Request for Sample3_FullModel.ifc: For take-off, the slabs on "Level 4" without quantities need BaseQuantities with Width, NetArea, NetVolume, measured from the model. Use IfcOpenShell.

First a look at what the model holds.

```python
import ifcopenshell
import ifcopenshell.util.element
import ifcopenshell.util.unit

model = ifcopenshell.open("Sample3_FullModel.ifc")
print(model.schema)
for unit_type in ("LENGTHUNIT", "AREAUNIT", "VOLUMEUNIT"):
    print(unit_type, ifcopenshell.util.unit.calculate_unit_scale(model, unit_type))
storey = next(s for s in model.by_type("IfcBuildingStorey") if s.Name == "Level 4")
slabs = [e for e in ifcopenshell.util.element.get_decomposition(storey) if e.is_a("IfcSlab")]
for e in sorted(slabs, key=lambda e: e.id()):
    print(e.id(), e.is_a(), e.Name, list(ifcopenshell.util.element.get_psets(e, qtos_only=True)), sep=" | ")
```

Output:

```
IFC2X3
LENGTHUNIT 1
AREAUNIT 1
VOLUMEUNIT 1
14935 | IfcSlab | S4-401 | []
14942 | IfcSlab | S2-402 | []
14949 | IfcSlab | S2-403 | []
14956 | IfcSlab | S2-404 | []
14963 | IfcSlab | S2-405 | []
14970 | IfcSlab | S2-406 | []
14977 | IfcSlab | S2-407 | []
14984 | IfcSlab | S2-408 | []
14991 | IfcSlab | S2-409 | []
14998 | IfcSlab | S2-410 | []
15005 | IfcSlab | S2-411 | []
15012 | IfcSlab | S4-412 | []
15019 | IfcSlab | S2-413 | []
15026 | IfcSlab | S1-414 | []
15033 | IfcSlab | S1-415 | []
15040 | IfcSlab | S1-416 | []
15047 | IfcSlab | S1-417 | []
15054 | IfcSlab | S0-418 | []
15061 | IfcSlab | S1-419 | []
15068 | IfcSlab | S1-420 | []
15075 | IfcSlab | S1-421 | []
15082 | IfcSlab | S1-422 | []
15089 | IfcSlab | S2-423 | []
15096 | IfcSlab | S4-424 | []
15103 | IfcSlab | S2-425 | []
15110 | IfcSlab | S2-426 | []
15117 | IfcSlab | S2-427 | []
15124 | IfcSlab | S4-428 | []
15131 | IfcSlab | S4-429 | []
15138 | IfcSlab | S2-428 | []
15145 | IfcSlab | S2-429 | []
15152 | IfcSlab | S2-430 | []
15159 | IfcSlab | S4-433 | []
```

```python
import ifcopenshell
import ifcopenshell.api.pset
import ifcopenshell.geom
import ifcopenshell.util.element
import ifcopenshell.util.shape
import ifcopenshell.util.unit

model = ifcopenshell.open("Sample3_FullModel.ifc")
unit_scale = ifcopenshell.util.unit.calculate_unit_scale(model)
area_scale = ifcopenshell.util.unit.calculate_unit_scale(model, "AREAUNIT")
volume_scale = ifcopenshell.util.unit.calculate_unit_scale(model, "VOLUMEUNIT")
settings = ifcopenshell.geom.settings()

storey = next(s for s in model.by_type("IfcBuildingStorey") if s.Name == "Level 4")
slabs = [e for e in ifcopenshell.util.element.get_decomposition(storey) if e.is_a("IfcSlab")]

for e in sorted(slabs, key=lambda e: e.id()):
    if ifcopenshell.util.element.get_psets(e, qtos_only=True, should_inherit=False):
        continue
    # Geometry comes back in metres, in the element's own axes.
    shape = ifcopenshell.geom.create_shape(settings, e)
    values = {
        "Width": ifcopenshell.util.shape.get_z(shape.geometry) / unit_scale,
        "NetArea": ifcopenshell.util.shape.get_footprint_area(shape.geometry) / area_scale,
        "NetVolume": ifcopenshell.util.shape.get_volume(shape.geometry) / volume_scale,
    }
    qto = ifcopenshell.api.pset.add_qto(model, product=e, name="BaseQuantities")
    ifcopenshell.api.pset.edit_qto(model, qto=qto, properties=values)
    print(e.id(), {k: round(v, 3) for k, v in values.items()})

model.write("Sample3_FullModel_updated.ifc")
```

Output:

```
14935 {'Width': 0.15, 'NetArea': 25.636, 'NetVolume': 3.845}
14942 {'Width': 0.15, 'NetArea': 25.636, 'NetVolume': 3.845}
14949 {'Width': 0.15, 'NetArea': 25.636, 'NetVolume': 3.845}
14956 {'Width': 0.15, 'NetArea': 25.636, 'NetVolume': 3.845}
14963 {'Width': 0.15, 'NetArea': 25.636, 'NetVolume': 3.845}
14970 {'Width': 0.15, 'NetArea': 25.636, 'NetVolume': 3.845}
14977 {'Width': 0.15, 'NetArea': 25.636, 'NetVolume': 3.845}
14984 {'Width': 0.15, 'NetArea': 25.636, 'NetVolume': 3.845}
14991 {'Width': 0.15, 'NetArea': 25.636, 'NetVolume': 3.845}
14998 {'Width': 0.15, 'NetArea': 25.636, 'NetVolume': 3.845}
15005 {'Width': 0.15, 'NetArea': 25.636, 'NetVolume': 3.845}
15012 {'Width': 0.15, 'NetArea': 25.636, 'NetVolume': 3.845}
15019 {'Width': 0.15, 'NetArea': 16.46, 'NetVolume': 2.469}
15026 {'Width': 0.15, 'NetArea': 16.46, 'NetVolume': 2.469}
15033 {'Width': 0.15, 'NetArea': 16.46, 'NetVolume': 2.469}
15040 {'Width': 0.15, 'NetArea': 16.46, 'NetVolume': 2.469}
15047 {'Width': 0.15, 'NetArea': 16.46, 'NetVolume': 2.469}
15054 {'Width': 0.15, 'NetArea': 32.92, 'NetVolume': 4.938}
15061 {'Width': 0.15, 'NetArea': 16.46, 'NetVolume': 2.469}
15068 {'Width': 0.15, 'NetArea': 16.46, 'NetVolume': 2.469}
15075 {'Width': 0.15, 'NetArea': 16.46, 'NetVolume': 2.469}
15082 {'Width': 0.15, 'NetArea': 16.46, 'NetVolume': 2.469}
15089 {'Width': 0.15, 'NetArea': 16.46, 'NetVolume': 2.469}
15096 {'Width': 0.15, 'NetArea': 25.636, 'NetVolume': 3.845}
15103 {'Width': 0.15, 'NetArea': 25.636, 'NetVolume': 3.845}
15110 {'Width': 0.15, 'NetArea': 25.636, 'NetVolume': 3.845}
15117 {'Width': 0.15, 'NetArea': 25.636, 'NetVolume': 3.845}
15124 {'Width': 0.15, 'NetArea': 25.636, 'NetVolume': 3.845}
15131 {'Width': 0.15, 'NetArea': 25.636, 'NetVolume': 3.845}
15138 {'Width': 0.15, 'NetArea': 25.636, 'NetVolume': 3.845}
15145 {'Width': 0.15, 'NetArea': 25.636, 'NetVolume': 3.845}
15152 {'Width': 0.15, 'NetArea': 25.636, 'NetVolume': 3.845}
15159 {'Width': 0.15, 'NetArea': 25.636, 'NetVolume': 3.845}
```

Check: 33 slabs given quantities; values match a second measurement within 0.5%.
